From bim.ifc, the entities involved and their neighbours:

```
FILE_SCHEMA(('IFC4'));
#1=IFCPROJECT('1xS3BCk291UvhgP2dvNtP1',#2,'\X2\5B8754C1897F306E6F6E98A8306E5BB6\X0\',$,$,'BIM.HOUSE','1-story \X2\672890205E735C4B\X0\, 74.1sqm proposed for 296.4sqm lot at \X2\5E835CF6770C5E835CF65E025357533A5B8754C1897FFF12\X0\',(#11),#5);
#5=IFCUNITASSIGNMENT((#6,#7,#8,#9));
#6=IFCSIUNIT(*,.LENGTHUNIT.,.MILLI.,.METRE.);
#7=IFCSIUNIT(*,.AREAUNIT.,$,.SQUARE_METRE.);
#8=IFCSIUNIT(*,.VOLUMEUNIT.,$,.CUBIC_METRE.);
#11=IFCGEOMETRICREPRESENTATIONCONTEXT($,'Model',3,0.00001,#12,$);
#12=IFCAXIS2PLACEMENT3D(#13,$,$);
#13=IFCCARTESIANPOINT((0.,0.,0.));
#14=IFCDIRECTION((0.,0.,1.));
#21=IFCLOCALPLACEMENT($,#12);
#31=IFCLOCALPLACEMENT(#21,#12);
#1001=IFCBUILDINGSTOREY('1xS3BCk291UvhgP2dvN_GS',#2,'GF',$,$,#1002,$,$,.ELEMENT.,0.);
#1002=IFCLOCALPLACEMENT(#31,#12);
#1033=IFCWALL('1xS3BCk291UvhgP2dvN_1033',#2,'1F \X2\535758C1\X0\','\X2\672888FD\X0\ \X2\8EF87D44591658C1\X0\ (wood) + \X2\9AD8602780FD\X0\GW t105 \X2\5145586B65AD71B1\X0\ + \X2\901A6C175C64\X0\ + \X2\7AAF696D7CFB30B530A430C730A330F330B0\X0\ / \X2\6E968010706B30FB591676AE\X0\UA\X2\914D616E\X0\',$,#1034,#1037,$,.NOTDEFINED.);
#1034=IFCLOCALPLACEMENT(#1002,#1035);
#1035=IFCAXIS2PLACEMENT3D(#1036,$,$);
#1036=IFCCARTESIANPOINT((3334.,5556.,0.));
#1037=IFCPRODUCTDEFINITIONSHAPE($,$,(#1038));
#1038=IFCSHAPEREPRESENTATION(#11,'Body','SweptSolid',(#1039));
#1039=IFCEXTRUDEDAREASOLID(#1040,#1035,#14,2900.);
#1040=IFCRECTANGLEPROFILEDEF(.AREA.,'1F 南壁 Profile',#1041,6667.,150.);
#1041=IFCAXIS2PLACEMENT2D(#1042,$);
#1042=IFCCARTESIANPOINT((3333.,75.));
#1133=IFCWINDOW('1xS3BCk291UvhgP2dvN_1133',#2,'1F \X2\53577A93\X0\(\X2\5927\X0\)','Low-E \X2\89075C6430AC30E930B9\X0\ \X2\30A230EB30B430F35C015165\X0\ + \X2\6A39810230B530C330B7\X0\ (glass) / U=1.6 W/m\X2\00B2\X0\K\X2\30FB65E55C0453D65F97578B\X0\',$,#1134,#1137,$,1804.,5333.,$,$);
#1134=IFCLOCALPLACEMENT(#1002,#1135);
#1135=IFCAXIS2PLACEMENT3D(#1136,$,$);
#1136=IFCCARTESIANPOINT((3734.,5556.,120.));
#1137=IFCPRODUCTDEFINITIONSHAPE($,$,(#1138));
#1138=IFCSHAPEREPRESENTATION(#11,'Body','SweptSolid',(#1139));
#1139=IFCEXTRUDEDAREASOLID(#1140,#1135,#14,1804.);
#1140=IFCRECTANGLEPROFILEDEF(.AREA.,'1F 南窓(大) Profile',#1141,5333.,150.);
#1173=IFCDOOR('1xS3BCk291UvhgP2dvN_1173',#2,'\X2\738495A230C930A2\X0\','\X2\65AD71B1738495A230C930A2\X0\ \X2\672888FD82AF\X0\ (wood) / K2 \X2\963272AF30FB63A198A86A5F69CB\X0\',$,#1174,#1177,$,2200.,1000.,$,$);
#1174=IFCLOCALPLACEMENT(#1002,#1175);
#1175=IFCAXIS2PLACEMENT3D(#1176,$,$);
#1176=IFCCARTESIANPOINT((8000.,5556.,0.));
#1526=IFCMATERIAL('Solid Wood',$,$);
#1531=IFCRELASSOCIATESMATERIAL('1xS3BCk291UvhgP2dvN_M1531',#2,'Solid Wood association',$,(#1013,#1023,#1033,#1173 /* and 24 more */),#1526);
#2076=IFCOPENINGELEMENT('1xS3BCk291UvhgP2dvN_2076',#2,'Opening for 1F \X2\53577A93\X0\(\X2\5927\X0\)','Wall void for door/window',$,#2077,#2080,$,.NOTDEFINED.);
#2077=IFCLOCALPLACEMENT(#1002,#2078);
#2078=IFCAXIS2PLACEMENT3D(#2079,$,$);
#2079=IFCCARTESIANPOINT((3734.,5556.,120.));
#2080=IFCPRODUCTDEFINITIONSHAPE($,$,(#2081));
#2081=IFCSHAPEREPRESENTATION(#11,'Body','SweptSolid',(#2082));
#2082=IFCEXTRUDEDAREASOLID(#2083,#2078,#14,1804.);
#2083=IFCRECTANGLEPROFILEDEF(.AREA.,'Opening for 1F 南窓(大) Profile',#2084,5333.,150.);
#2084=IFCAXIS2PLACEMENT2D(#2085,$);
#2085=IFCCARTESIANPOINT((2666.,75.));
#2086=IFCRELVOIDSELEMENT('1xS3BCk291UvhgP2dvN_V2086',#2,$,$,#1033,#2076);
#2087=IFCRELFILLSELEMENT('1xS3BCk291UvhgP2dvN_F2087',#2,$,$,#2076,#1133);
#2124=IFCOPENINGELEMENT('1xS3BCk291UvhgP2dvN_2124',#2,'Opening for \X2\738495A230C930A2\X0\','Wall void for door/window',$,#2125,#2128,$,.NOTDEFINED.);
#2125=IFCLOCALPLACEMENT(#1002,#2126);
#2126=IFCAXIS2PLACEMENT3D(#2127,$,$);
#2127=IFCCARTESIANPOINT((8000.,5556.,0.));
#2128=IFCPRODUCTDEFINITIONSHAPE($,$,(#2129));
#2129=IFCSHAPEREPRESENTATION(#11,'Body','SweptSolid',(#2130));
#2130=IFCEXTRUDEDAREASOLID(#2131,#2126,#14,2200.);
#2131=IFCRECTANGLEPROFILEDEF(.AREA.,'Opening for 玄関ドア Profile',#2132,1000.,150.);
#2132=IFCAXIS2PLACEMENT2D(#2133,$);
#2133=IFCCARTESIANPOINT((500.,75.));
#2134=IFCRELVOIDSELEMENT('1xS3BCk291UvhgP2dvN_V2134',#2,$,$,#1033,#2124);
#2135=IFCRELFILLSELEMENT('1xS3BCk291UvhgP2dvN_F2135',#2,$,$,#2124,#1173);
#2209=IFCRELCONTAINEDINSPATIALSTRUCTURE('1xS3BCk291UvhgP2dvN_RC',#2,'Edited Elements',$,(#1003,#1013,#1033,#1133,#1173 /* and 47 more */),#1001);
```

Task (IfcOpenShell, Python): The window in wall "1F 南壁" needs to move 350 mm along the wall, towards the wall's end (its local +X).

```python
import ifcopenshell
import ifcopenshell.api.geometry
import ifcopenshell.util.placement

model = ifcopenshell.open("bim.ifc")

window = model.by_guid("1xS3BCk291UvhgP2dvN_1133")
opening = window.FillsVoids[0].RelatingOpeningElement
wall = opening.VoidsElements[0].RelatingBuildingElement

wall_matrix = ifcopenshell.util.placement.get_local_placement(wall.ObjectPlacement)
shift = wall_matrix[:3, 0] * 350.0
before = ifcopenshell.util.placement.get_local_placement(window.ObjectPlacement)[:3, 3].copy()

# The window is not placed relative to its opening, so move both.
for product in (opening, window):
    matrix = ifcopenshell.util.placement.get_local_placement(product.ObjectPlacement)
    matrix[:3, 3] += shift
    ifcopenshell.api.geometry.edit_object_placement(model, product=product, matrix=matrix, is_si=False)

after = ifcopenshell.util.placement.get_local_placement(window.ObjectPlacement)[:3, 3]
print("window moved by", (after - before).round(3) + 0.0)

model.write("bim_edited.ifc")
```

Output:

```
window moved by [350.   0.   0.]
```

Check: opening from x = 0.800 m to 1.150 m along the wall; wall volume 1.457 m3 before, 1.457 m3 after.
